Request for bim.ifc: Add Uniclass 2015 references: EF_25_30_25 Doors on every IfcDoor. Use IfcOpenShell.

First a look at what the model holds.

```python
import ifcopenshell

model = ifcopenshell.open("bim.ifc")
print(model.schema)
print("classifications:", [c.Name for c in model.by_type("IfcClassification")])
for ifc_class in ("IfcDoor", "IfcRoof", "IfcStair", "IfcWall", "IfcWindow"):
    print(ifc_class, len(model.by_type(ifc_class)))
```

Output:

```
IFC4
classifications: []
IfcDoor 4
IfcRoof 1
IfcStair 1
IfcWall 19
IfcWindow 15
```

```python
import ifcopenshell
import ifcopenshell.api.classification

model = ifcopenshell.open("bim.ifc")

system = ifcopenshell.api.classification.add_classification(model, classification="Uniclass 2015")

codes = {
    "IfcDoor": ("EF_25_30_25", "Doors"),
}
for ifc_class, (code, name) in codes.items():
    products = model.by_type(ifc_class)
    ifcopenshell.api.classification.add_reference(
        model, products=products, classification=system, identification=code, name=name
    )
    print(code, len(products))

model.write("bim_updated.ifc")
```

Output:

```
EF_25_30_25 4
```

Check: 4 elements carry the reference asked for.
